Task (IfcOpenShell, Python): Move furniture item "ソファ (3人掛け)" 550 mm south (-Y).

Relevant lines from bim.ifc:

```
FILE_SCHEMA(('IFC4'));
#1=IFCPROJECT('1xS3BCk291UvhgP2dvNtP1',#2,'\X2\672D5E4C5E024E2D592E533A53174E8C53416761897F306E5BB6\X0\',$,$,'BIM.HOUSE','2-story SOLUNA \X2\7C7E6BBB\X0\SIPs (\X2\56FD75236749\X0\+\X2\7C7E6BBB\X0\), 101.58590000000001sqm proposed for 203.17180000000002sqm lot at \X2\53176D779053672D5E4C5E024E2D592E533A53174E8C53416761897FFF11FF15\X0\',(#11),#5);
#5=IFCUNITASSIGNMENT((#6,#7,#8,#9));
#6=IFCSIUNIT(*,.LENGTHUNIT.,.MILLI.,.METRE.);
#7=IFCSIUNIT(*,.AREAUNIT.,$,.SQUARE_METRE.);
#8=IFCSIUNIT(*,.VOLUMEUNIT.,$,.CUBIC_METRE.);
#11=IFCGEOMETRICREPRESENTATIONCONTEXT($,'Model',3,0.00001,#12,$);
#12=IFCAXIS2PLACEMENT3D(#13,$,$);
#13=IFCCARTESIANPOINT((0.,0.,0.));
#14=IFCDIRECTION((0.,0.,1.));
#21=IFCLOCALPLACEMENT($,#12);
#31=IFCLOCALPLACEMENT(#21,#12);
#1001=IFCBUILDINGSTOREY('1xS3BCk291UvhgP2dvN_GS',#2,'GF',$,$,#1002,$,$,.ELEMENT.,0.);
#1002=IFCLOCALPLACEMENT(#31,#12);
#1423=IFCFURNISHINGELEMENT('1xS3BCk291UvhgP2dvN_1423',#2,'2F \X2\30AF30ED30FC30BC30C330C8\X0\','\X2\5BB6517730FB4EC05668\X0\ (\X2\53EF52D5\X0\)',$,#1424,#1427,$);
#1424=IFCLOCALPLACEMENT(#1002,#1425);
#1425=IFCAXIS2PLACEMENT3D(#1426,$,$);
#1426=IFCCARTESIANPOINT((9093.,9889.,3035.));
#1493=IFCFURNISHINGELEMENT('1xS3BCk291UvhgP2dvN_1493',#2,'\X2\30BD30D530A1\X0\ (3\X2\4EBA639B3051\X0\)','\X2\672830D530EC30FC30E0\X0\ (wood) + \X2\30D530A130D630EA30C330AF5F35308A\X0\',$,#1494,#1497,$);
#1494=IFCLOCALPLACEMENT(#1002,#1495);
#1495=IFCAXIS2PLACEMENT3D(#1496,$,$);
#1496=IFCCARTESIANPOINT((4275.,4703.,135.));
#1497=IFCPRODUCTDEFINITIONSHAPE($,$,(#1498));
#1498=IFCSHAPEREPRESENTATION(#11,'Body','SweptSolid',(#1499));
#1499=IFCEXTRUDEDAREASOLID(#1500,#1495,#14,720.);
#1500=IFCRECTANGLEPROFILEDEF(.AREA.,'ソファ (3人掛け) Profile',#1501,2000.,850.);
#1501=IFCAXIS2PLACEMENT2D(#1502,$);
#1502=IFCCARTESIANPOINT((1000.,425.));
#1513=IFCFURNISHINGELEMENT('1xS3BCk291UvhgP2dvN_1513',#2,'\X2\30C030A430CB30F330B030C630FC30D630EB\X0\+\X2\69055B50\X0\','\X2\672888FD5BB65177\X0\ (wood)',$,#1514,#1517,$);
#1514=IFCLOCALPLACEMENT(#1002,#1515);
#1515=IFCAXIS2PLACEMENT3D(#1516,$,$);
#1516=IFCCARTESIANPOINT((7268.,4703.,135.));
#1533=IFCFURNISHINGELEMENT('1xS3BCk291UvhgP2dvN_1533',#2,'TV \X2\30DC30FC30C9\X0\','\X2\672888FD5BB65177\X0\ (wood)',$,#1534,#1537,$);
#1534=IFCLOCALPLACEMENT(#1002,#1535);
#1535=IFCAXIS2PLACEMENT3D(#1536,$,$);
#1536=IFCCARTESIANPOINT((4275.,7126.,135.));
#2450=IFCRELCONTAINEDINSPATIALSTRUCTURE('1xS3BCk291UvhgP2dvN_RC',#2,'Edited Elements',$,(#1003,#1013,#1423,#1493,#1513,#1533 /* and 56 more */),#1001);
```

```python
import ifcopenshell
import ifcopenshell.api.geometry
import ifcopenshell.util.placement
import ifcopenshell.util.unit

model = ifcopenshell.open("bim.ifc")
unit_scale = ifcopenshell.util.unit.calculate_unit_scale(model)

item = model.by_id(1493)
matrix = ifcopenshell.util.placement.get_local_placement(item.ObjectPlacement)
matrix[1, 3] -= 0.55 / unit_scale
ifcopenshell.api.geometry.edit_object_placement(model, product=item, matrix=matrix, is_si=False)

print(ifcopenshell.util.placement.get_local_placement(item.ObjectPlacement).round(3) + 0.0)

model.write("bim_v2.ifc")
```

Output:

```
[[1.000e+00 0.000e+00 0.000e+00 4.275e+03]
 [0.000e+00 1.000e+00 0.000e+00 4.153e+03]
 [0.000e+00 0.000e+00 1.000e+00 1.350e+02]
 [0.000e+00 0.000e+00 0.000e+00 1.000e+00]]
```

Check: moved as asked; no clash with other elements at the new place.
